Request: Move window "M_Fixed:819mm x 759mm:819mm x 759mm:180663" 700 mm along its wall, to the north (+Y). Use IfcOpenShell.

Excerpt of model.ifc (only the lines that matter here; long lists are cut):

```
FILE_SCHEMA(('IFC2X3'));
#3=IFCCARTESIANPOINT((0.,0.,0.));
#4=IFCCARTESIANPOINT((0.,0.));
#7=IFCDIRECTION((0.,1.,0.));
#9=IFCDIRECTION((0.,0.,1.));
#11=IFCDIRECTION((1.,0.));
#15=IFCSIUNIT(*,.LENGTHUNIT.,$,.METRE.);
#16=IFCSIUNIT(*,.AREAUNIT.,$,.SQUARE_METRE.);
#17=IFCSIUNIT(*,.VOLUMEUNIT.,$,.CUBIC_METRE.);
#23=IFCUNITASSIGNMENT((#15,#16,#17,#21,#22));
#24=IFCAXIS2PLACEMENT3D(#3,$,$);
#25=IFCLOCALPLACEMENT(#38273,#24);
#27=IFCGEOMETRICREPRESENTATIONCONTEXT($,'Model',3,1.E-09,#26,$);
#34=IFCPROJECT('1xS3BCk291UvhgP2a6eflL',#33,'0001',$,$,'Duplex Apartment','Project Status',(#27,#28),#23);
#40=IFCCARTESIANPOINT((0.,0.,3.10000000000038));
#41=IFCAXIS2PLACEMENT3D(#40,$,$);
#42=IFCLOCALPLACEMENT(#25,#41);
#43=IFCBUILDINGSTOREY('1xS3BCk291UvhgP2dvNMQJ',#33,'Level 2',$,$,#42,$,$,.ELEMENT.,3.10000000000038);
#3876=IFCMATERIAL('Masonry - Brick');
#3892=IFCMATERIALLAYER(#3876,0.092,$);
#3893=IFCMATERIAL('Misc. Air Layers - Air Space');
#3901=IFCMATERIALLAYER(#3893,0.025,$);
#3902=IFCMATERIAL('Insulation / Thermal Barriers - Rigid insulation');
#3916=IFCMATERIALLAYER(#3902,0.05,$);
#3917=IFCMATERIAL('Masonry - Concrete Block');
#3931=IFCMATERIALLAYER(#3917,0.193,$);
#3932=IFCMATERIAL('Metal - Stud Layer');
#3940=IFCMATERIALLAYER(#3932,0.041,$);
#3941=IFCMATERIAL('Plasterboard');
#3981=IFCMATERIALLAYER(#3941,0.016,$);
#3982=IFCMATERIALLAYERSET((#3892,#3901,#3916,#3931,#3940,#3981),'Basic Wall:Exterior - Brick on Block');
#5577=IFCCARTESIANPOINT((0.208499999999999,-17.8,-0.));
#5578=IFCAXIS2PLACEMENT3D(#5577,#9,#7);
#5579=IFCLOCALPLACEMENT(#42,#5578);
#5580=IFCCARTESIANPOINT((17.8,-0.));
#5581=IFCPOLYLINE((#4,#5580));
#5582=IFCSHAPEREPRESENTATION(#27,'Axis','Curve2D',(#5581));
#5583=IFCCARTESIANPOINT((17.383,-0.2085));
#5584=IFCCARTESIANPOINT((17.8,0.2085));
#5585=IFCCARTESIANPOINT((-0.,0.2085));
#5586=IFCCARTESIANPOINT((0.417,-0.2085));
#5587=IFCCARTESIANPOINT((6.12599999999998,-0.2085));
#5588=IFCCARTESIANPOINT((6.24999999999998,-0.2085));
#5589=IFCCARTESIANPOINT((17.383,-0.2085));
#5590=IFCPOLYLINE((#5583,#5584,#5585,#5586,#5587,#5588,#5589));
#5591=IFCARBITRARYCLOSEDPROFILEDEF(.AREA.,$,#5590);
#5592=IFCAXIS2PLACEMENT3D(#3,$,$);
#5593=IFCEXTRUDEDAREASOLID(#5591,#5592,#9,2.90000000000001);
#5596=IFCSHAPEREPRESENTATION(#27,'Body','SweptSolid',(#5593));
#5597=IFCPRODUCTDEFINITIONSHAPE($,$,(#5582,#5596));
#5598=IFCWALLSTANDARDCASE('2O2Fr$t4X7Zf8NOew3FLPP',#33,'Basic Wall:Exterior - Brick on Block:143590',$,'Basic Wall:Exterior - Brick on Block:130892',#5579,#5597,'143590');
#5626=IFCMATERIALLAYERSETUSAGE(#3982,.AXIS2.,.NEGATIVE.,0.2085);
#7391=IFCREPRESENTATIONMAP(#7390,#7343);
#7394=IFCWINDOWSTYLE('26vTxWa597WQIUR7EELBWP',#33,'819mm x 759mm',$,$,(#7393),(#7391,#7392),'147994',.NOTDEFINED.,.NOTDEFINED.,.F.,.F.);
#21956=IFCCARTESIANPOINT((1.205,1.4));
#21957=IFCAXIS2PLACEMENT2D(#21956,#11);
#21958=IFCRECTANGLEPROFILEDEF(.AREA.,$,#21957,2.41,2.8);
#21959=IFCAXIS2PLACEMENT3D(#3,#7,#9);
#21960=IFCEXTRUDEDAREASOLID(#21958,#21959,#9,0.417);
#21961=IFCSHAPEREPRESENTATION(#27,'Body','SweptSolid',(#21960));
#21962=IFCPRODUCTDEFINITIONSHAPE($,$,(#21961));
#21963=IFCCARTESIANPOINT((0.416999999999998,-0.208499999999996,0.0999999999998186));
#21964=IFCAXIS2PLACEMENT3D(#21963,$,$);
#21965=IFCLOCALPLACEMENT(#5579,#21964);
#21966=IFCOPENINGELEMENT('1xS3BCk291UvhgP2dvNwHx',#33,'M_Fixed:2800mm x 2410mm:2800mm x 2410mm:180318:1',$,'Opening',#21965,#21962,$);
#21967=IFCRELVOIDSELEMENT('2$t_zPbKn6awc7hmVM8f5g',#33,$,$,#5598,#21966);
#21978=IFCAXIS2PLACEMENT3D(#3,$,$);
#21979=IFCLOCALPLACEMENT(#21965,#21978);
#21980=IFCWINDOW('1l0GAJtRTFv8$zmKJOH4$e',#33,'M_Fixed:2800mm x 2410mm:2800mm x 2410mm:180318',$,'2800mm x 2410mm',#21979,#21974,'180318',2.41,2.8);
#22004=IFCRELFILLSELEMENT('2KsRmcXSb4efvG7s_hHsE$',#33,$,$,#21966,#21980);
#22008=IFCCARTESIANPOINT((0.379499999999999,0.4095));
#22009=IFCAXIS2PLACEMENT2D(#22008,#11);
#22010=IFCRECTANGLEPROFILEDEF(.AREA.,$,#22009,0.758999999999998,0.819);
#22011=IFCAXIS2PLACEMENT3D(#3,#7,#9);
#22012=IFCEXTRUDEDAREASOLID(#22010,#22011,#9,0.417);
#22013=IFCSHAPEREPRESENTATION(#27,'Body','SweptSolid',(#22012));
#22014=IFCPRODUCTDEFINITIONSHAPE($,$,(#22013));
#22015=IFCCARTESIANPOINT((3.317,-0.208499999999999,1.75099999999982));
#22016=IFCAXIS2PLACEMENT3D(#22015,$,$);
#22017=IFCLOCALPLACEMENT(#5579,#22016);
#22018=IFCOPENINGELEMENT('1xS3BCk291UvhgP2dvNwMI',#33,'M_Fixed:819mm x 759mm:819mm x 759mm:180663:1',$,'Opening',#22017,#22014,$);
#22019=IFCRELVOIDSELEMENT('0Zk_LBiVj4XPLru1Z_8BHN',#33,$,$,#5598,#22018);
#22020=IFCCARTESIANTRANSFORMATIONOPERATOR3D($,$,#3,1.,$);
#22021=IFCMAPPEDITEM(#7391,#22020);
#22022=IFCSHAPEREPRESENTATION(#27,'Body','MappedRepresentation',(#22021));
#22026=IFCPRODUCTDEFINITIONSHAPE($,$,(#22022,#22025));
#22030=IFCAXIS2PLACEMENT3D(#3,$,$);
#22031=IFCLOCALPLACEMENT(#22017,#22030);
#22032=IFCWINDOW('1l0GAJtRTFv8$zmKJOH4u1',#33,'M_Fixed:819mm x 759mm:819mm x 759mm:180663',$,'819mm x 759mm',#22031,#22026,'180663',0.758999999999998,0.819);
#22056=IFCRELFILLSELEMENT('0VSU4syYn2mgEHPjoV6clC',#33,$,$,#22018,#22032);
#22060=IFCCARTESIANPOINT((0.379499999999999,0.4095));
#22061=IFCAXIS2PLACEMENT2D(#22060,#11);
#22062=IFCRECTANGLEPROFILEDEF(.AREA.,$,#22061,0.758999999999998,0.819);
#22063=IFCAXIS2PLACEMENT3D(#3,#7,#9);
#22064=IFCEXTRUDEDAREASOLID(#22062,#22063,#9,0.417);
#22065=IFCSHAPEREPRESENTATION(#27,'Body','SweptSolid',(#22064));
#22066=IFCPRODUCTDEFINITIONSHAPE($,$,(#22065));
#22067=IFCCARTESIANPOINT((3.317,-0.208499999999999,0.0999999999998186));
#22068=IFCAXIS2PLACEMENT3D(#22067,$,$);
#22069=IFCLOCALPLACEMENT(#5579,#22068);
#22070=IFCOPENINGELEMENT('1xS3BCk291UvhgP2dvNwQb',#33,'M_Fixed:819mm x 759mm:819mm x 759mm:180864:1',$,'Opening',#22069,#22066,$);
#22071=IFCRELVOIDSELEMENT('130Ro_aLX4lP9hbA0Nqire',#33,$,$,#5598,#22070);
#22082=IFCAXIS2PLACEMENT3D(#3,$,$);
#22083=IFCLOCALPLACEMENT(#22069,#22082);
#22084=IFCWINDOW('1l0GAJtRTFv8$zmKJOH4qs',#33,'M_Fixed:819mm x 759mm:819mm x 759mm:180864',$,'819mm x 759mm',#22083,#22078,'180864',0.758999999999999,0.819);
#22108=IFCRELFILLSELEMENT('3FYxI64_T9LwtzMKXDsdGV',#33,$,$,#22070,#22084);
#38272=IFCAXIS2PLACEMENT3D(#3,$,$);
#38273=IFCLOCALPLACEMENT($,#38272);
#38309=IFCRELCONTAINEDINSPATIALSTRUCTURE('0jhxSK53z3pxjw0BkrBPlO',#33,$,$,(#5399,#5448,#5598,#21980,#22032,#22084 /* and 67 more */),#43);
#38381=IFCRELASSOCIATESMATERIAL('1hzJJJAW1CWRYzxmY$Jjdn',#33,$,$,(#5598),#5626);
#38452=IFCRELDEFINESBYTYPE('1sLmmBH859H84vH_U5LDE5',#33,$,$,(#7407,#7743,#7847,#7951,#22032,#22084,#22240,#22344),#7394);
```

```python
import ifcopenshell
import ifcopenshell.api.geometry
import ifcopenshell.util.placement

model = ifcopenshell.open("model.ifc")

window = model.by_guid("1l0GAJtRTFv8$zmKJOH4u1")
opening = window.FillsVoids[0].RelatingOpeningElement
wall = opening.VoidsElements[0].RelatingBuildingElement

wall_matrix = ifcopenshell.util.placement.get_local_placement(wall.ObjectPlacement)
shift = wall_matrix[:3, 0] * 0.7
before = ifcopenshell.util.placement.get_local_placement(window.ObjectPlacement)[:3, 3].copy()

# The window is placed relative to its opening, so it follows when the opening moves.
matrix = ifcopenshell.util.placement.get_local_placement(opening.ObjectPlacement)
matrix[:3, 3] += shift
ifcopenshell.api.geometry.edit_object_placement(
    model, product=opening, matrix=matrix, is_si=False, should_transform_children=True
)

after = ifcopenshell.util.placement.get_local_placement(window.ObjectPlacement)[:3, 3]
print("window moved by", (after - before).round(3) + 0.0)

model.write("model-out.ifc")
```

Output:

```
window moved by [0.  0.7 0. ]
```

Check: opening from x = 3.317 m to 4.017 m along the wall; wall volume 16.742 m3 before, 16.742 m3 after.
